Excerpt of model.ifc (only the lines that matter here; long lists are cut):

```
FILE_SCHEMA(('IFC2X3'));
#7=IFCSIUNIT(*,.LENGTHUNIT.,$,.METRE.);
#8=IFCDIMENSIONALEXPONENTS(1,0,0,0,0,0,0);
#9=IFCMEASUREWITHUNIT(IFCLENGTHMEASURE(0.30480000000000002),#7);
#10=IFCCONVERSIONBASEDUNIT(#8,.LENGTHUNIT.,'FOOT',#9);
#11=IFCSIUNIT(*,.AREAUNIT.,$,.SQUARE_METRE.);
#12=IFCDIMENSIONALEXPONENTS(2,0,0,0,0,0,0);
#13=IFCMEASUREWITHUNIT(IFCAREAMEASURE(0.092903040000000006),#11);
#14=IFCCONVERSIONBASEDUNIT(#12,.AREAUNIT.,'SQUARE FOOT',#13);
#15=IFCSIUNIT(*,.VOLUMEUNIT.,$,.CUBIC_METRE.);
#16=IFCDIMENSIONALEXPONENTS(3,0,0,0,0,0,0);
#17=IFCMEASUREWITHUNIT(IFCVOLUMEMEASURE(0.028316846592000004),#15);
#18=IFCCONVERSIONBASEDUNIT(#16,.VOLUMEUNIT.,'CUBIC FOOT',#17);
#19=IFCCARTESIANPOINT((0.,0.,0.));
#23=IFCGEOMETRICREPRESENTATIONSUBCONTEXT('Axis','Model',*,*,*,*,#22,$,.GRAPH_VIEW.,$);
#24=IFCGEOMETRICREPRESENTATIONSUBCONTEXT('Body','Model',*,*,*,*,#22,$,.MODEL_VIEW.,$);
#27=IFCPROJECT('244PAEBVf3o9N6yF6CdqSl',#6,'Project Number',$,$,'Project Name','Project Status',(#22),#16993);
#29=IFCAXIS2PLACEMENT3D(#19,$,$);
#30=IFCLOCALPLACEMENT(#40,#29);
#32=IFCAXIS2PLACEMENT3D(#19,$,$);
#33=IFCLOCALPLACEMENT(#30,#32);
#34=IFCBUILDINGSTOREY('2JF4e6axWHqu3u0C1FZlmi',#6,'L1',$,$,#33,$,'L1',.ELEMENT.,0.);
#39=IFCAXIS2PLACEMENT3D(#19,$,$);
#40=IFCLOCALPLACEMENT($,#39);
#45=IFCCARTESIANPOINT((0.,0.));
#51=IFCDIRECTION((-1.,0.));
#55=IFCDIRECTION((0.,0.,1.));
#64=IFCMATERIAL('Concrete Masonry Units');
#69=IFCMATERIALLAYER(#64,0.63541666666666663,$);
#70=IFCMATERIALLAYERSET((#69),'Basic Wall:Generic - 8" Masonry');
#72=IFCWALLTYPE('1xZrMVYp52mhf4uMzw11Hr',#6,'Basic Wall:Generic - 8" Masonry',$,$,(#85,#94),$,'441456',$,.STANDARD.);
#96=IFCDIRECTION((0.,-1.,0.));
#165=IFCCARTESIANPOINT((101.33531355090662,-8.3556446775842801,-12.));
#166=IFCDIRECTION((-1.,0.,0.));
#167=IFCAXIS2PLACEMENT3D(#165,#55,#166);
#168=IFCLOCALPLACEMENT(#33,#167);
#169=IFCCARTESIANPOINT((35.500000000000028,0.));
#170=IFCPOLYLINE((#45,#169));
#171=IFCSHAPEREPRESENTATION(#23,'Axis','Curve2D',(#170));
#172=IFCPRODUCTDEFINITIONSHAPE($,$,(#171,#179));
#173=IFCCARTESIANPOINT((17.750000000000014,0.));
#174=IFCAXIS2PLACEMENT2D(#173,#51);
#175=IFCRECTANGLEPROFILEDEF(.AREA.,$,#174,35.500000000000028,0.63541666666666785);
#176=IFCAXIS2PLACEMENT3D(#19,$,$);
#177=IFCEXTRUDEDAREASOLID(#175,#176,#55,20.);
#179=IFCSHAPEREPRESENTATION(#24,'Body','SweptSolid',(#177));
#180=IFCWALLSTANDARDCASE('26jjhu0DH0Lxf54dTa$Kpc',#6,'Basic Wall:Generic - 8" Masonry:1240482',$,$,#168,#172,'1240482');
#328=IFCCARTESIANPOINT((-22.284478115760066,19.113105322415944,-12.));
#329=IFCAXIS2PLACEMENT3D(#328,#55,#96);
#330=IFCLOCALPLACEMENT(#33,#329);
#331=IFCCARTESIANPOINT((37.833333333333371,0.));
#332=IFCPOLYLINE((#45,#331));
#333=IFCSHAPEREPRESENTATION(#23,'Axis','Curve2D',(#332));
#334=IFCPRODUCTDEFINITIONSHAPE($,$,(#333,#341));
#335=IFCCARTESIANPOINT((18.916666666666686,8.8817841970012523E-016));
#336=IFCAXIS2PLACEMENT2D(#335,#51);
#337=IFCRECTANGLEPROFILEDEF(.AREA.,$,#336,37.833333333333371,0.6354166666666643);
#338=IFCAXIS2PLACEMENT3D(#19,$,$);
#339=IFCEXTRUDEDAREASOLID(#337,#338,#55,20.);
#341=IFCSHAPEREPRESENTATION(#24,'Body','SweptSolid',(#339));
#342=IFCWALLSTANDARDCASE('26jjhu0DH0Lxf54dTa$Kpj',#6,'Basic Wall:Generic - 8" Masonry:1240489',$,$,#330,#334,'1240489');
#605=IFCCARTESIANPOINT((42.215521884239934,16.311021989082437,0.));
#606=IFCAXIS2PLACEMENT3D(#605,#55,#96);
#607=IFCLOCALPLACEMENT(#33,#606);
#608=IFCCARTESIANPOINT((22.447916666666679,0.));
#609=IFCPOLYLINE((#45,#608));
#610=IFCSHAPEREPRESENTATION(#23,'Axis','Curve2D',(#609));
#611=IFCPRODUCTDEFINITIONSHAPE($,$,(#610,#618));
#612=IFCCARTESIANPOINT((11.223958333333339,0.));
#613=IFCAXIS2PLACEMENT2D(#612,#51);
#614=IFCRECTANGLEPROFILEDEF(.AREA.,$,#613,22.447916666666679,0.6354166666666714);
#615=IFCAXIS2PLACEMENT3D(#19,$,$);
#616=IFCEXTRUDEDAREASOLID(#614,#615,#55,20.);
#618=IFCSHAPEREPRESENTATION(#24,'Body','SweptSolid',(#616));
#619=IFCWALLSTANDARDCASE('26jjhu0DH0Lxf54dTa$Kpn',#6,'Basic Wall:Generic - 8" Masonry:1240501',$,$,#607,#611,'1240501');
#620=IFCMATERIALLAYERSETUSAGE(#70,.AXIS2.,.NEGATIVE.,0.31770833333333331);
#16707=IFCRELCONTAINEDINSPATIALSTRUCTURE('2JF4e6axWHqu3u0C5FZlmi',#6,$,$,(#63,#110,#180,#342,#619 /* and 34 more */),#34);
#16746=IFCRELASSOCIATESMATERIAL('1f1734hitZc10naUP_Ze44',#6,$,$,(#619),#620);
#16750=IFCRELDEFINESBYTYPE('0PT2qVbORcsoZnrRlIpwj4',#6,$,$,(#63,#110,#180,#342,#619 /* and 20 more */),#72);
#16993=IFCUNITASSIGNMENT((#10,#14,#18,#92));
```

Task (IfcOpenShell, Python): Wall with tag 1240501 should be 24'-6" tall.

```python
import ifcopenshell
import ifcopenshell.geom
import ifcopenshell.util.representation
import ifcopenshell.util.shape
import ifcopenshell.util.unit

model = ifcopenshell.open("model.ifc")
unit_scale = ifcopenshell.util.unit.calculate_unit_scale(model)
settings = ifcopenshell.geom.settings()


def volume(element):
    """Net volume in cubic metres, openings subtracted."""
    shape = ifcopenshell.geom.create_shape(settings, element)
    return ifcopenshell.util.shape.get_volume(shape.geometry)


wall = model.by_id(619)
before = volume(wall)

body = ifcopenshell.util.representation.get_representation(wall, "Model", "Body")
solid = body.Items[0]
old_height = solid.Depth
solid.Depth = 294 * 0.0254 / unit_scale
after = volume(wall)

print(f"height {old_height:g} -> {solid.Depth:g}, volume {before:.3f} -> {after:.3f} m3")

model.write("model_edited.ifc")
```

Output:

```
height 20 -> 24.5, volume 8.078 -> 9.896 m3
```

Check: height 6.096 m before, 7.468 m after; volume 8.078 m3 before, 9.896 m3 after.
